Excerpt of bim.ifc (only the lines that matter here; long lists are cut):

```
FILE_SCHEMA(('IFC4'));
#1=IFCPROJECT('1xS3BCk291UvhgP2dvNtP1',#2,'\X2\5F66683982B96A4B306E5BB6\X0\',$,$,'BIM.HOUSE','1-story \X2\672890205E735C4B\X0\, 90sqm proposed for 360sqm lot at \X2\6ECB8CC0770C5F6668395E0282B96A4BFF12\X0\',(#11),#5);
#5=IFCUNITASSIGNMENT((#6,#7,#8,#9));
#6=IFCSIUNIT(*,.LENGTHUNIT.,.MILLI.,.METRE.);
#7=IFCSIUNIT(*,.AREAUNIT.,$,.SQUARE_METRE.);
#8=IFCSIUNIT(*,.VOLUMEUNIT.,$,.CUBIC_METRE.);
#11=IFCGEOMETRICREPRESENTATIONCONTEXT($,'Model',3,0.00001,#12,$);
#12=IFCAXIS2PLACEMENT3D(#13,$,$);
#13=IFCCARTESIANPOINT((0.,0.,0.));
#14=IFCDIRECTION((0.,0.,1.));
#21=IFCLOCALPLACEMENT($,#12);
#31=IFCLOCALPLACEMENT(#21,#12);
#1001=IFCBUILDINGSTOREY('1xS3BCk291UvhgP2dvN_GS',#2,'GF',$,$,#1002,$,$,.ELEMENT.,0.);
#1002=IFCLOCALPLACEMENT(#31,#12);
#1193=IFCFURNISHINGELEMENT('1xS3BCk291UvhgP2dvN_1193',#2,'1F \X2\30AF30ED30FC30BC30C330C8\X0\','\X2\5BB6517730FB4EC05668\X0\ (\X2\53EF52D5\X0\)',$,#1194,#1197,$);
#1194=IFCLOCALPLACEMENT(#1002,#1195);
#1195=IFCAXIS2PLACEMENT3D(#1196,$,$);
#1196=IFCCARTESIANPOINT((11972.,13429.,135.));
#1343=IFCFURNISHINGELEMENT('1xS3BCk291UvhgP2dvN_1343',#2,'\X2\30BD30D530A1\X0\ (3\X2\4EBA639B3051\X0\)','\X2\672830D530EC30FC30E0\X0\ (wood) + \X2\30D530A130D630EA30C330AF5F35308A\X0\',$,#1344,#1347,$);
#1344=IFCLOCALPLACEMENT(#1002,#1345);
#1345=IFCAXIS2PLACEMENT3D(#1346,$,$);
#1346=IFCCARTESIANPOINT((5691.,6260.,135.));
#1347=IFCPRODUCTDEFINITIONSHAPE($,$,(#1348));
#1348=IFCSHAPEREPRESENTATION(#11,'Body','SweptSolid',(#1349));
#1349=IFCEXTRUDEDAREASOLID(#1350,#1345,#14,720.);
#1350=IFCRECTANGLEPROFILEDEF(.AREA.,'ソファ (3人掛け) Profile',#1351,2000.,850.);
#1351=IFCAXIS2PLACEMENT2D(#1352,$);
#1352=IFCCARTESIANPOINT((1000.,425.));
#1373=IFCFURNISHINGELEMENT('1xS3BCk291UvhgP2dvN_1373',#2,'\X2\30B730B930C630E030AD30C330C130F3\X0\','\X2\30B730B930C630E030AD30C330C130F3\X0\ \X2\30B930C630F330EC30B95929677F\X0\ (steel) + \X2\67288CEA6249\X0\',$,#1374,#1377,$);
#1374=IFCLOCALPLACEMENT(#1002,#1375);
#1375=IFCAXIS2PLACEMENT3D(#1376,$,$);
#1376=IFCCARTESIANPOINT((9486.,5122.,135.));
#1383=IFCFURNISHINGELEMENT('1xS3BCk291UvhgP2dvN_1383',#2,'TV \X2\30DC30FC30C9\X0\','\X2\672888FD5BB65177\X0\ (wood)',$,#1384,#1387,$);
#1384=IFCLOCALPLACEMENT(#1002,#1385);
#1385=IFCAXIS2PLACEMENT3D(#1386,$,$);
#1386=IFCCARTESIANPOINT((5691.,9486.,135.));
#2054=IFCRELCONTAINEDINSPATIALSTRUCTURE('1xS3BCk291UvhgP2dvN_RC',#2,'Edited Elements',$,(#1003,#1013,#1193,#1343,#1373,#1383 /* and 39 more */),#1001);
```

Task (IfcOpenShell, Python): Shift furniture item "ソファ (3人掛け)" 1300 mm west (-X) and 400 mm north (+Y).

```python
import ifcopenshell
import ifcopenshell.api.geometry
import ifcopenshell.util.placement

model = ifcopenshell.open("bim.ifc")

item = model.by_id(1343)
matrix = ifcopenshell.util.placement.get_local_placement(item.ObjectPlacement)
matrix[0, 3] -= 1300.0
matrix[1, 3] += 400.0
ifcopenshell.api.geometry.edit_object_placement(model, product=item, matrix=matrix, is_si=False)

print(ifcopenshell.util.placement.get_local_placement(item.ObjectPlacement).round(3) + 0.0)

model.write("bim-out.ifc")
```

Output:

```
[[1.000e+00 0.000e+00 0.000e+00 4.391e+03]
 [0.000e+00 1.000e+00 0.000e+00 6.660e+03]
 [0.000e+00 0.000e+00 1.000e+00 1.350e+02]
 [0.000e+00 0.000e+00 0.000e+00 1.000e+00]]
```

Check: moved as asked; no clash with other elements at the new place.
